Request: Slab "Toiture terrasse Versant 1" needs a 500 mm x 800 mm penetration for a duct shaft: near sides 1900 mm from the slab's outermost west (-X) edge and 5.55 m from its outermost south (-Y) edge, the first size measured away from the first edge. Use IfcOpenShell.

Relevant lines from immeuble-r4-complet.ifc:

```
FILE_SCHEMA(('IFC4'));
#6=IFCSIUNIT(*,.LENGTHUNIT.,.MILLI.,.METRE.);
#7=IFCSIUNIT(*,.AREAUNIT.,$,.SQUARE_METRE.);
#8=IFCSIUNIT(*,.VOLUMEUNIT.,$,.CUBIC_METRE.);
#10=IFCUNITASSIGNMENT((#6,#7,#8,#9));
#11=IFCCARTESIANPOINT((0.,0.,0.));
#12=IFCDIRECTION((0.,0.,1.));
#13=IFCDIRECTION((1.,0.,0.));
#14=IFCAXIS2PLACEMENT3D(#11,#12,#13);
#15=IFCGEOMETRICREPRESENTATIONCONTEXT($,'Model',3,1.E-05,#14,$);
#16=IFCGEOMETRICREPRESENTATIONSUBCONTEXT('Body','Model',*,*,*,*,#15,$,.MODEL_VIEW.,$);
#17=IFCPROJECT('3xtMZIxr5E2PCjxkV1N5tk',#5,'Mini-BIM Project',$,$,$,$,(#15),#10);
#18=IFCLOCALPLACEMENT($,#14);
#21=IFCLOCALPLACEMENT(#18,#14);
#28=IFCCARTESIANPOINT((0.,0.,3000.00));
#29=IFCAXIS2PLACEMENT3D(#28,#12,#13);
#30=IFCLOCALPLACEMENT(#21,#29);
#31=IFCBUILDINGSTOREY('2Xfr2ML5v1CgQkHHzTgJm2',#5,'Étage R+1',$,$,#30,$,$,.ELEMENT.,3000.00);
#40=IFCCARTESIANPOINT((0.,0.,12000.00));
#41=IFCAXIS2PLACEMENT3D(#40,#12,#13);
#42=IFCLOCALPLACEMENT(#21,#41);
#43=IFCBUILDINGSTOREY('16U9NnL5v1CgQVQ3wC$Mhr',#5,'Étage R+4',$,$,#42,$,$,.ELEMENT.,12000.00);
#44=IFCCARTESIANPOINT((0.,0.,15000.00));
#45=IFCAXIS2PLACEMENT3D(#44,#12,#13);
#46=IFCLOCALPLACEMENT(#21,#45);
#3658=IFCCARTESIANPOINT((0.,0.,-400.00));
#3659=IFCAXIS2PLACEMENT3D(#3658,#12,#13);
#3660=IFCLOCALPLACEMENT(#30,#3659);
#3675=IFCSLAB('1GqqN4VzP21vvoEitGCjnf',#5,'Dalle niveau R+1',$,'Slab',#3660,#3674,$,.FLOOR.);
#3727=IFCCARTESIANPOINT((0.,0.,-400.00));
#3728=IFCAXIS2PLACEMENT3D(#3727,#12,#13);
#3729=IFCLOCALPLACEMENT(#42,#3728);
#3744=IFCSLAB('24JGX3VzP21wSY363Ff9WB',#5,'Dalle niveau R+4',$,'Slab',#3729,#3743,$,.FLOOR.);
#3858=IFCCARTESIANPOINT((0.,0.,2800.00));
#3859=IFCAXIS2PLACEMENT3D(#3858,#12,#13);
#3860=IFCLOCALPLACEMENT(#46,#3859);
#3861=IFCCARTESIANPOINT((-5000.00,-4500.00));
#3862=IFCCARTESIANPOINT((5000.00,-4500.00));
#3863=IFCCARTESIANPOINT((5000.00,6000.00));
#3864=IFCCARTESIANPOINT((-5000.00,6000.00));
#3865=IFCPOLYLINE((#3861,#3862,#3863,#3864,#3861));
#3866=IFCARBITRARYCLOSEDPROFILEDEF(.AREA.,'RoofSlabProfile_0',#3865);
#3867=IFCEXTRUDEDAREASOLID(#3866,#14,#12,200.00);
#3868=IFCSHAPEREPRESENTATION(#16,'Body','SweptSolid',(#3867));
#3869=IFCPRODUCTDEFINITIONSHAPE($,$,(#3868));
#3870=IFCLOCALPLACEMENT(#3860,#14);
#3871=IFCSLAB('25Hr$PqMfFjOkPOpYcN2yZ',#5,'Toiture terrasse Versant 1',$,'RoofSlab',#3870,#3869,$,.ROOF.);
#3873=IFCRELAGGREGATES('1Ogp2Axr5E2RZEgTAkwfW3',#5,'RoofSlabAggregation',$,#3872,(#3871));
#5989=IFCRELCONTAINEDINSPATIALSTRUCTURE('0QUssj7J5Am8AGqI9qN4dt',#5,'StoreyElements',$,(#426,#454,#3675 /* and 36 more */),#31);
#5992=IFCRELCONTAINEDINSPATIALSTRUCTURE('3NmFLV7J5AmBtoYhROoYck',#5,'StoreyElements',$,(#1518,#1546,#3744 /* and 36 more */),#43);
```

```python
import numpy as np
import ifcopenshell
import ifcopenshell.api.feature
import ifcopenshell.api.geometry
import ifcopenshell.api.root
import ifcopenshell.geom
import ifcopenshell.util.placement
import ifcopenshell.util.representation
import ifcopenshell.util.shape
import ifcopenshell.util.unit

model = ifcopenshell.open("immeuble-r4-complet.ifc")
unit_scale = ifcopenshell.util.unit.calculate_unit_scale(model)
settings = ifcopenshell.geom.settings()


def volume(element):
    """Net volume in cubic metres, openings subtracted."""
    shape = ifcopenshell.geom.create_shape(settings, element)
    return ifcopenshell.util.shape.get_volume(shape.geometry)


slab = model.by_guid("25Hr$PqMfFjOkPOpYcN2yZ")
before = volume(slab)

# Extent in the slab's own axes, in metres. The edges named are its -X and -Y sides.
slab_shape = ifcopenshell.geom.create_shape(settings, slab)
vertices = ifcopenshell.util.shape.get_vertices(slab_shape.geometry)
x_min, y_min, bottom = vertices.min(axis=0)
top = vertices[:, 2].max()

opening = ifcopenshell.api.root.create_entity(model, ifc_class="IfcOpeningElement", name="Duct shaft opening", predefined_type="OPENING")
context = ifcopenshell.util.representation.get_context(model, "Model", "Body", "MODEL_VIEW")
width, depth = 0.5, 0.8
outline = [(0.0, 0.0), (width, 0.0), (width, depth), (0.0, depth), (0.0, 0.0)]
# Overshoot both faces by 50 mm so the cut is clean.
shape = ifcopenshell.api.geometry.add_slab_representation(
    model, context=context, depth=top - bottom + 0.1, polyline=outline
)
ifcopenshell.api.geometry.assign_representation(model, product=opening, representation=shape)

matrix = ifcopenshell.util.placement.get_local_placement(slab.ObjectPlacement)
matrix[:, 3] = matrix @ np.append(np.array([x_min + 1.9, y_min + 5.55, bottom - 0.05]) / unit_scale, 1.0)
ifcopenshell.api.geometry.edit_object_placement(model, product=opening, matrix=matrix, is_si=False)
ifcopenshell.api.feature.add_feature(model, feature=opening, element=slab)

after = volume(slab)

print(f"slab volume {before:.3f} -> {after:.3f} m3")

model.write("immeuble-r4-complet_rev.ifc")
```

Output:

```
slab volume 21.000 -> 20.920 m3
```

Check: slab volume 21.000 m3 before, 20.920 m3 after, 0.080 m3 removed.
